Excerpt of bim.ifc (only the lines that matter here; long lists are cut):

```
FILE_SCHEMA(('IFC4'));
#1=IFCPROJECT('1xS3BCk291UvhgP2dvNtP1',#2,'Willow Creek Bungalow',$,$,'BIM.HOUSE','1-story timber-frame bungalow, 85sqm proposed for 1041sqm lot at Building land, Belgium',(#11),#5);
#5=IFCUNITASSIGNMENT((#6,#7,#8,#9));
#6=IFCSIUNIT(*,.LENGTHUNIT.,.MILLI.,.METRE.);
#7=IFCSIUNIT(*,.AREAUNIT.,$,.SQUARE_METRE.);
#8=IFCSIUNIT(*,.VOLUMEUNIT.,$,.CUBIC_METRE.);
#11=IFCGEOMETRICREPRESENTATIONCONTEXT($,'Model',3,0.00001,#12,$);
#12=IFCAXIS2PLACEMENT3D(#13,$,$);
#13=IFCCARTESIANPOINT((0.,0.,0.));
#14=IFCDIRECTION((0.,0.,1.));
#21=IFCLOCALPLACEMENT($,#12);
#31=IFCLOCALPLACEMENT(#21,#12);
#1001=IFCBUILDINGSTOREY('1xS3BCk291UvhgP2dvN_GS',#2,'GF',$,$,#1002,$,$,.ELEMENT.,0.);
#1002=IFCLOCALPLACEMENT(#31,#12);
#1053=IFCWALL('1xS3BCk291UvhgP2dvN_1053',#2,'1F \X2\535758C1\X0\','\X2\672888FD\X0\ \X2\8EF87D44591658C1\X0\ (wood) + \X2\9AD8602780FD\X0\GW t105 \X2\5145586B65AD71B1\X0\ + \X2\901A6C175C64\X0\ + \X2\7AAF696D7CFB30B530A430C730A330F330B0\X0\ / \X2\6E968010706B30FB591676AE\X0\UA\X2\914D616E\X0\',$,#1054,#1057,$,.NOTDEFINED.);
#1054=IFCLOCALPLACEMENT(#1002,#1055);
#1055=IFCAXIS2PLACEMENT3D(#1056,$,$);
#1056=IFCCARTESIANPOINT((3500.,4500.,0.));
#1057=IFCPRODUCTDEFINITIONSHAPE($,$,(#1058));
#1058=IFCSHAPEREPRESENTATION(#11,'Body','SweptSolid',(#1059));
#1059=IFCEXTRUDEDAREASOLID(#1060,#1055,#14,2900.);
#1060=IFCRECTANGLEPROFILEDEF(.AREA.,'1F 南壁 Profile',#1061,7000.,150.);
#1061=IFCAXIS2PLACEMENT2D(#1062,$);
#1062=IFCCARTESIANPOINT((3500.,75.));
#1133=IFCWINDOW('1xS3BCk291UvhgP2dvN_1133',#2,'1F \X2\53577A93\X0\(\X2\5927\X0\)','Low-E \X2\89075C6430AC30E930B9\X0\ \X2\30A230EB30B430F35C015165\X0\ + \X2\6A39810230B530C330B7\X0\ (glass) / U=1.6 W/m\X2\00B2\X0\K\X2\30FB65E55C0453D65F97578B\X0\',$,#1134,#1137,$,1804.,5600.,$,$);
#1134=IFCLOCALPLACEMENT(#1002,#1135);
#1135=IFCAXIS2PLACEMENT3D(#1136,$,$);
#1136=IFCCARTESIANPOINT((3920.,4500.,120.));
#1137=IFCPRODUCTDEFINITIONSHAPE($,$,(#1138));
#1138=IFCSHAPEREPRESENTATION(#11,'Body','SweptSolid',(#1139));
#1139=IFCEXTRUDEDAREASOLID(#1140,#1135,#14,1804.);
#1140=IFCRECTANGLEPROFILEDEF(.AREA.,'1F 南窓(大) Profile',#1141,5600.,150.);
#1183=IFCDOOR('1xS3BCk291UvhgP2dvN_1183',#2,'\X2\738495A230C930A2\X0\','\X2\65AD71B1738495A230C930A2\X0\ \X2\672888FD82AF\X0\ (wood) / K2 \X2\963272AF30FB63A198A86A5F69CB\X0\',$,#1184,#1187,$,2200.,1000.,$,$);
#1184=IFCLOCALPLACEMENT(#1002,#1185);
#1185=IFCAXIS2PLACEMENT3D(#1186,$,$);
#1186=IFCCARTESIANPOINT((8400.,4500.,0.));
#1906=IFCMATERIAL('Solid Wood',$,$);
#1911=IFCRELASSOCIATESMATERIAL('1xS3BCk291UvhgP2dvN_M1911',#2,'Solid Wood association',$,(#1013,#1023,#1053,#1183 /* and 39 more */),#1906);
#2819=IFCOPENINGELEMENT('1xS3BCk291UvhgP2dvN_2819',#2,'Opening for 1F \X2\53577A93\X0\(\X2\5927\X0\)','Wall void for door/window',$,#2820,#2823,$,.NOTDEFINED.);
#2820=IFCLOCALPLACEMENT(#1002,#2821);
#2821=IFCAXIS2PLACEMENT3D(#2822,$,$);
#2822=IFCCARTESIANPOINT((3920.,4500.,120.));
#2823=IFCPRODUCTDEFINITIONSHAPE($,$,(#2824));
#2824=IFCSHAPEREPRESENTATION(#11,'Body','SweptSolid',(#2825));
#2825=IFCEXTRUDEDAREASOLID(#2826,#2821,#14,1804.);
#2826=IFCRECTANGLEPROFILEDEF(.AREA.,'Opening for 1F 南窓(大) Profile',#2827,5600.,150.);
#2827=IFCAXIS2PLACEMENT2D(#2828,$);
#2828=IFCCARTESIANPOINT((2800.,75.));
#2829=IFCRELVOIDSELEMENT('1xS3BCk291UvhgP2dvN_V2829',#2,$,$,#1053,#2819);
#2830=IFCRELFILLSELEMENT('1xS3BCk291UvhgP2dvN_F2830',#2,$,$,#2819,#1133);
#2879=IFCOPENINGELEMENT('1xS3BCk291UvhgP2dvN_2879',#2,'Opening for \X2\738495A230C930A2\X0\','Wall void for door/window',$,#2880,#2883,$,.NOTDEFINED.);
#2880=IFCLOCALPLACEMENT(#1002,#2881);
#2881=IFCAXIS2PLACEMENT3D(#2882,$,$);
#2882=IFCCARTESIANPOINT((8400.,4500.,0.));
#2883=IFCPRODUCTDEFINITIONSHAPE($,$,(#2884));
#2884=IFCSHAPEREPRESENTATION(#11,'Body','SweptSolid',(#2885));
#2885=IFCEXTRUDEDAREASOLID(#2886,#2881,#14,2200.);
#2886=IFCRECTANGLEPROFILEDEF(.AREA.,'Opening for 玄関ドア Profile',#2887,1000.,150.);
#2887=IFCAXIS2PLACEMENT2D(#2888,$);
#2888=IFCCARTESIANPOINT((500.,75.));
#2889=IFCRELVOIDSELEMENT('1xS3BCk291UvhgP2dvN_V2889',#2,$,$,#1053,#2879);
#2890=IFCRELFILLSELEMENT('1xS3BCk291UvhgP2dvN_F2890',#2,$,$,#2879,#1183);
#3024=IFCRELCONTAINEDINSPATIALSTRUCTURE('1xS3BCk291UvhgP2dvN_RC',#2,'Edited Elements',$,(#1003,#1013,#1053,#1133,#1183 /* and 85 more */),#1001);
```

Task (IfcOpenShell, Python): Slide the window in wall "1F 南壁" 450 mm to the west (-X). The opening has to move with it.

```python
import ifcopenshell
import ifcopenshell.api.geometry
import ifcopenshell.util.placement

model = ifcopenshell.open("bim.ifc")

window = model.by_guid("1xS3BCk291UvhgP2dvN_1133")
opening = window.FillsVoids[0].RelatingOpeningElement
wall = opening.VoidsElements[0].RelatingBuildingElement

wall_matrix = ifcopenshell.util.placement.get_local_placement(wall.ObjectPlacement)
shift = wall_matrix[:3, 0] * -450.0
before = ifcopenshell.util.placement.get_local_placement(window.ObjectPlacement)[:3, 3].copy()

# The window is not placed relative to its opening, so move both.
for product in (opening, window):
    matrix = ifcopenshell.util.placement.get_local_placement(product.ObjectPlacement)
    matrix[:3, 3] += shift
    ifcopenshell.api.geometry.edit_object_placement(model, product=product, matrix=matrix, is_si=False)

after = ifcopenshell.util.placement.get_local_placement(window.ObjectPlacement)[:3, 3]
print("window moved by", (after - before).round(3) + 0.0)

model.write("bim_edited.ifc")
```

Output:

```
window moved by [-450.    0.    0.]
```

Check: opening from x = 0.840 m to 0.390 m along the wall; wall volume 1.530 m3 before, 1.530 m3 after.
